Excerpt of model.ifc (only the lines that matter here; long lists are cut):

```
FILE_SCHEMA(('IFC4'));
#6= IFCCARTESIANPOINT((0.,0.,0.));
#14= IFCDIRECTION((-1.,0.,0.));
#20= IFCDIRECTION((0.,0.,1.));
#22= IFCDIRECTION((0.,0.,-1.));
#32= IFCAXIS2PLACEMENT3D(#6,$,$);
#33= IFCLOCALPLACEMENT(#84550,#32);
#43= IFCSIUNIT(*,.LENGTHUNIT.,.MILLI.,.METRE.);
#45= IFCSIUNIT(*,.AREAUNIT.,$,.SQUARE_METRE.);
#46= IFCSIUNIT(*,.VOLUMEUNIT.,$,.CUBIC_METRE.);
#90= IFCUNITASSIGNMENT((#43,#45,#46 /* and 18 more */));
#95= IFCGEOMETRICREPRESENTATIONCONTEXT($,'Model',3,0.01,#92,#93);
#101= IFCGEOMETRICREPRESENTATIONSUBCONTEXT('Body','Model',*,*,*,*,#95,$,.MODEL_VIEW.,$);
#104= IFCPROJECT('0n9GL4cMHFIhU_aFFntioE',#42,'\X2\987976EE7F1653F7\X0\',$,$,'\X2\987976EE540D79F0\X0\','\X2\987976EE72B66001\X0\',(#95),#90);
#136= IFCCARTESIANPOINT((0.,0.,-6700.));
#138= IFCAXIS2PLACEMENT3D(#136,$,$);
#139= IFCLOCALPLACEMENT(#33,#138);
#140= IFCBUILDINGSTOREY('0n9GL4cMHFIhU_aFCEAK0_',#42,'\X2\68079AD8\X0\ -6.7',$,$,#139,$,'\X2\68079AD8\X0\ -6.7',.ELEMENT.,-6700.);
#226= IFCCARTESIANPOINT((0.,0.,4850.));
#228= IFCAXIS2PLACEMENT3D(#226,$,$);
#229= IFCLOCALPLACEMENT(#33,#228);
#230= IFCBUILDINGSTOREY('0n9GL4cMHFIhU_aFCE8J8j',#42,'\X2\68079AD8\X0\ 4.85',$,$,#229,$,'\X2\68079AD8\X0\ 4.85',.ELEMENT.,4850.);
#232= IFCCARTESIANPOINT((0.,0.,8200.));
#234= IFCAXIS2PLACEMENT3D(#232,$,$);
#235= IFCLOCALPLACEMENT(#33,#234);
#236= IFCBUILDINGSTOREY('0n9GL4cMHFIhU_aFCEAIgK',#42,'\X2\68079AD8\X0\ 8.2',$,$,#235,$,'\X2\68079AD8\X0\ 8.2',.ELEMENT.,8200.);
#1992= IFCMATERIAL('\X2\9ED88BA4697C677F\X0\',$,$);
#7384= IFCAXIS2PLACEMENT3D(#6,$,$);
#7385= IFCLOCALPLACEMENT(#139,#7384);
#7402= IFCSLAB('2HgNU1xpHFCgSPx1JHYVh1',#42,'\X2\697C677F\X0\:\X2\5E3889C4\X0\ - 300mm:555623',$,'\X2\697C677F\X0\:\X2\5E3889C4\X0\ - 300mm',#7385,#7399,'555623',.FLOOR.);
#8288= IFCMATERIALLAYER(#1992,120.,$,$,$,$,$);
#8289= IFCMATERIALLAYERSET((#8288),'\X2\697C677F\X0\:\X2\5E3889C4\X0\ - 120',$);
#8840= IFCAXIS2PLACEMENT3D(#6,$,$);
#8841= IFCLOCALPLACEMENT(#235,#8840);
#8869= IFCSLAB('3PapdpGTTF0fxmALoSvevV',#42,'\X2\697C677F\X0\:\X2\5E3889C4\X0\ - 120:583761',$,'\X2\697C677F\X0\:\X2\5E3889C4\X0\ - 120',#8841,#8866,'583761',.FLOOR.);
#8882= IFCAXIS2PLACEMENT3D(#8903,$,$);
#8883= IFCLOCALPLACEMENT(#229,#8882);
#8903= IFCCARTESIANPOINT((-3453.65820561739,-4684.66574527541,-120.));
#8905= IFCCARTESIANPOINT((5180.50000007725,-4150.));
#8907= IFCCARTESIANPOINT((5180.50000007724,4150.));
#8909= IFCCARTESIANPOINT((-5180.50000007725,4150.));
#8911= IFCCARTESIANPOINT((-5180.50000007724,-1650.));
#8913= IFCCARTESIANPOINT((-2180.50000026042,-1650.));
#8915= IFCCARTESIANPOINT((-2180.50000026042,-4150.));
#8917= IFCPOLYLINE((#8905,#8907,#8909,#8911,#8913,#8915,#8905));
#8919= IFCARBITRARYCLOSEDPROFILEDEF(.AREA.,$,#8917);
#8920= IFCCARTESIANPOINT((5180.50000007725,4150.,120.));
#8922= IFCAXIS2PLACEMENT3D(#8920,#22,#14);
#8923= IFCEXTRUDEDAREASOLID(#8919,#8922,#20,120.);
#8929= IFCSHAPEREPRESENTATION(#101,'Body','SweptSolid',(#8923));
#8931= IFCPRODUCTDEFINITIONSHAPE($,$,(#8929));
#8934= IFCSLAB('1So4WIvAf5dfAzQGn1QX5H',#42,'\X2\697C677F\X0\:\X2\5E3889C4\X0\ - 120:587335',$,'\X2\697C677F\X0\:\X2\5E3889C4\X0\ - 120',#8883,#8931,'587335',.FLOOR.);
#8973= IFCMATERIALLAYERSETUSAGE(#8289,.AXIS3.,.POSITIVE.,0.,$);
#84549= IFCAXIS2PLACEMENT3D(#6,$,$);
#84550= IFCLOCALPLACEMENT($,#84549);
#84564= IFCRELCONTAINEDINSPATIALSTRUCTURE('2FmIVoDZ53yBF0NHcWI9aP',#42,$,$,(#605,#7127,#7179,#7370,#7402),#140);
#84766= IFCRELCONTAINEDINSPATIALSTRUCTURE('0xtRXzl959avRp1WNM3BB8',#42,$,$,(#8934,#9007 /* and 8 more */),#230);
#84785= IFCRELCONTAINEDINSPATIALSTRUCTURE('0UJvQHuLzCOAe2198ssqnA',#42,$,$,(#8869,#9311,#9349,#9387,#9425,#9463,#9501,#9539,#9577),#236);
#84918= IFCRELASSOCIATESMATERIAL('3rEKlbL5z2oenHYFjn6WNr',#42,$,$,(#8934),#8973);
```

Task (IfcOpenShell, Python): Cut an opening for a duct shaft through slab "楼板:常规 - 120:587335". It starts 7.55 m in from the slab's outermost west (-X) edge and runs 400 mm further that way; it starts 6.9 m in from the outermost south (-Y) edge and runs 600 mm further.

```python
import numpy as np
import ifcopenshell
import ifcopenshell.api.feature
import ifcopenshell.api.geometry
import ifcopenshell.api.root
import ifcopenshell.geom
import ifcopenshell.util.placement
import ifcopenshell.util.representation
import ifcopenshell.util.shape
import ifcopenshell.util.unit

model = ifcopenshell.open("model.ifc")
unit_scale = ifcopenshell.util.unit.calculate_unit_scale(model)
settings = ifcopenshell.geom.settings()


def volume(element):
    """Net volume in cubic metres, openings subtracted."""
    shape = ifcopenshell.geom.create_shape(settings, element)
    return ifcopenshell.util.shape.get_volume(shape.geometry)


slab = model.by_guid("1So4WIvAf5dfAzQGn1QX5H")
before = volume(slab)

# Extent in the slab's own axes, in metres. The edges named are its -X and -Y sides.
slab_shape = ifcopenshell.geom.create_shape(settings, slab)
vertices = ifcopenshell.util.shape.get_vertices(slab_shape.geometry)
x_min, y_min, bottom = vertices.min(axis=0)
top = vertices[:, 2].max()

opening = ifcopenshell.api.root.create_entity(model, ifc_class="IfcOpeningElement", name="Duct shaft opening", predefined_type="OPENING")
context = ifcopenshell.util.representation.get_context(model, "Model", "Body", "MODEL_VIEW")
width, depth = 0.4, 0.6
outline = [(0.0, 0.0), (width, 0.0), (width, depth), (0.0, depth), (0.0, 0.0)]
# Overshoot both faces by 50 mm so the cut is clean.
shape = ifcopenshell.api.geometry.add_slab_representation(
    model, context=context, depth=top - bottom + 0.1, polyline=outline
)
ifcopenshell.api.geometry.assign_representation(model, product=opening, representation=shape)

matrix = ifcopenshell.util.placement.get_local_placement(slab.ObjectPlacement)
matrix[:, 3] = matrix @ np.append(np.array([x_min + 7.55, y_min + 6.9, bottom - 0.05]) / unit_scale, 1.0)
ifcopenshell.api.geometry.edit_object_placement(model, product=opening, matrix=matrix, is_si=False)
ifcopenshell.api.feature.add_feature(model, feature=opening, element=slab)

after = volume(slab)

print(f"slab volume {before:.3f} -> {after:.3f} m3")

model.write("model_updated.ifc")
```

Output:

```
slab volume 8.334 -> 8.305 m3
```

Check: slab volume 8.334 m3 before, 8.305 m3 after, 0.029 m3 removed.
